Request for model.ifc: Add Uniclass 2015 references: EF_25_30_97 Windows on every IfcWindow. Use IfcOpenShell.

First a look at what the model holds.

```python
import ifcopenshell

model = ifcopenshell.open("model.ifc")
print(model.schema)
print("classifications:", [c.Name for c in model.by_type("IfcClassification")])
for ifc_class in ("IfcDoor", "IfcRoof", "IfcStair", "IfcWall", "IfcWindow"):
    print(ifc_class, len(model.by_type(ifc_class)))
```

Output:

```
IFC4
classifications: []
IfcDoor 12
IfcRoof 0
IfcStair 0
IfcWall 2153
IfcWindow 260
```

```python
import ifcopenshell
import ifcopenshell.api.classification

model = ifcopenshell.open("model.ifc")

system = ifcopenshell.api.classification.add_classification(model, classification="Uniclass 2015")

codes = {
    "IfcWindow": ("EF_25_30_97", "Windows"),
}
for ifc_class, (code, name) in codes.items():
    products = model.by_type(ifc_class)
    ifcopenshell.api.classification.add_reference(
        model, products=products, classification=system, identification=code, name=name
    )
    print(code, len(products))

model.write("model_rev.ifc")
```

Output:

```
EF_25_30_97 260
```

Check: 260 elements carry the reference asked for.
